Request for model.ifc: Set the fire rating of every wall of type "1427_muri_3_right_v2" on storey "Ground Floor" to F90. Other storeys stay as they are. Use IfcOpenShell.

First a look at what the model holds.

```python
import ifcopenshell
import ifcopenshell.util.element

model = ifcopenshell.open("model.ifc")
print(model.schema)
storey = next(s for s in model.by_type("IfcBuildingStorey") if s.Name == "Ground Floor")
walls = [e for e in ifcopenshell.util.element.get_decomposition(storey) if e.is_a("IfcWall")]
seen = {}
for e in walls:
    element_type = ifcopenshell.util.element.get_type(e)
    key = (element_type.Name if element_type != e and element_type else None, ifcopenshell.util.element.get_pset(e, "Pset_WallCommon", "FireRating"))
    seen[key] = seen.get(key, 0) + 1
for (name, value), count in sorted(seen.items(), key=str):
    print(count, "x", name, "|", value)
```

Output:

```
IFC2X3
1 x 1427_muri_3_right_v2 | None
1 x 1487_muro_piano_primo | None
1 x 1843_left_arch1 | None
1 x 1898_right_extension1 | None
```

```python
import ifcopenshell
import ifcopenshell.api.pset
import ifcopenshell.util.element

model = ifcopenshell.open("model.ifc")

storey = next(s for s in model.by_type("IfcBuildingStorey") if s.Name == "Ground Floor")
walls = [e for e in ifcopenshell.util.element.get_decomposition(storey) if e.is_a("IfcWall")]

count = 0
for e in walls:
    element_type = ifcopenshell.util.element.get_type(e)
    if element_type in (None, e) or element_type.Name != "1427_muri_3_right_v2":
        continue
    # add_pset returns the element's existing set when there is one.
    pset = ifcopenshell.api.pset.add_pset(model, product=e, name="Pset_WallCommon")
    ifcopenshell.api.pset.edit_pset(model, pset=pset, properties={"FireRating": "F90"})
    count += 1

print(count, "walls updated")

model.write("model_v2.ifc")
```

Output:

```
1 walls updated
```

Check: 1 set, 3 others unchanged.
